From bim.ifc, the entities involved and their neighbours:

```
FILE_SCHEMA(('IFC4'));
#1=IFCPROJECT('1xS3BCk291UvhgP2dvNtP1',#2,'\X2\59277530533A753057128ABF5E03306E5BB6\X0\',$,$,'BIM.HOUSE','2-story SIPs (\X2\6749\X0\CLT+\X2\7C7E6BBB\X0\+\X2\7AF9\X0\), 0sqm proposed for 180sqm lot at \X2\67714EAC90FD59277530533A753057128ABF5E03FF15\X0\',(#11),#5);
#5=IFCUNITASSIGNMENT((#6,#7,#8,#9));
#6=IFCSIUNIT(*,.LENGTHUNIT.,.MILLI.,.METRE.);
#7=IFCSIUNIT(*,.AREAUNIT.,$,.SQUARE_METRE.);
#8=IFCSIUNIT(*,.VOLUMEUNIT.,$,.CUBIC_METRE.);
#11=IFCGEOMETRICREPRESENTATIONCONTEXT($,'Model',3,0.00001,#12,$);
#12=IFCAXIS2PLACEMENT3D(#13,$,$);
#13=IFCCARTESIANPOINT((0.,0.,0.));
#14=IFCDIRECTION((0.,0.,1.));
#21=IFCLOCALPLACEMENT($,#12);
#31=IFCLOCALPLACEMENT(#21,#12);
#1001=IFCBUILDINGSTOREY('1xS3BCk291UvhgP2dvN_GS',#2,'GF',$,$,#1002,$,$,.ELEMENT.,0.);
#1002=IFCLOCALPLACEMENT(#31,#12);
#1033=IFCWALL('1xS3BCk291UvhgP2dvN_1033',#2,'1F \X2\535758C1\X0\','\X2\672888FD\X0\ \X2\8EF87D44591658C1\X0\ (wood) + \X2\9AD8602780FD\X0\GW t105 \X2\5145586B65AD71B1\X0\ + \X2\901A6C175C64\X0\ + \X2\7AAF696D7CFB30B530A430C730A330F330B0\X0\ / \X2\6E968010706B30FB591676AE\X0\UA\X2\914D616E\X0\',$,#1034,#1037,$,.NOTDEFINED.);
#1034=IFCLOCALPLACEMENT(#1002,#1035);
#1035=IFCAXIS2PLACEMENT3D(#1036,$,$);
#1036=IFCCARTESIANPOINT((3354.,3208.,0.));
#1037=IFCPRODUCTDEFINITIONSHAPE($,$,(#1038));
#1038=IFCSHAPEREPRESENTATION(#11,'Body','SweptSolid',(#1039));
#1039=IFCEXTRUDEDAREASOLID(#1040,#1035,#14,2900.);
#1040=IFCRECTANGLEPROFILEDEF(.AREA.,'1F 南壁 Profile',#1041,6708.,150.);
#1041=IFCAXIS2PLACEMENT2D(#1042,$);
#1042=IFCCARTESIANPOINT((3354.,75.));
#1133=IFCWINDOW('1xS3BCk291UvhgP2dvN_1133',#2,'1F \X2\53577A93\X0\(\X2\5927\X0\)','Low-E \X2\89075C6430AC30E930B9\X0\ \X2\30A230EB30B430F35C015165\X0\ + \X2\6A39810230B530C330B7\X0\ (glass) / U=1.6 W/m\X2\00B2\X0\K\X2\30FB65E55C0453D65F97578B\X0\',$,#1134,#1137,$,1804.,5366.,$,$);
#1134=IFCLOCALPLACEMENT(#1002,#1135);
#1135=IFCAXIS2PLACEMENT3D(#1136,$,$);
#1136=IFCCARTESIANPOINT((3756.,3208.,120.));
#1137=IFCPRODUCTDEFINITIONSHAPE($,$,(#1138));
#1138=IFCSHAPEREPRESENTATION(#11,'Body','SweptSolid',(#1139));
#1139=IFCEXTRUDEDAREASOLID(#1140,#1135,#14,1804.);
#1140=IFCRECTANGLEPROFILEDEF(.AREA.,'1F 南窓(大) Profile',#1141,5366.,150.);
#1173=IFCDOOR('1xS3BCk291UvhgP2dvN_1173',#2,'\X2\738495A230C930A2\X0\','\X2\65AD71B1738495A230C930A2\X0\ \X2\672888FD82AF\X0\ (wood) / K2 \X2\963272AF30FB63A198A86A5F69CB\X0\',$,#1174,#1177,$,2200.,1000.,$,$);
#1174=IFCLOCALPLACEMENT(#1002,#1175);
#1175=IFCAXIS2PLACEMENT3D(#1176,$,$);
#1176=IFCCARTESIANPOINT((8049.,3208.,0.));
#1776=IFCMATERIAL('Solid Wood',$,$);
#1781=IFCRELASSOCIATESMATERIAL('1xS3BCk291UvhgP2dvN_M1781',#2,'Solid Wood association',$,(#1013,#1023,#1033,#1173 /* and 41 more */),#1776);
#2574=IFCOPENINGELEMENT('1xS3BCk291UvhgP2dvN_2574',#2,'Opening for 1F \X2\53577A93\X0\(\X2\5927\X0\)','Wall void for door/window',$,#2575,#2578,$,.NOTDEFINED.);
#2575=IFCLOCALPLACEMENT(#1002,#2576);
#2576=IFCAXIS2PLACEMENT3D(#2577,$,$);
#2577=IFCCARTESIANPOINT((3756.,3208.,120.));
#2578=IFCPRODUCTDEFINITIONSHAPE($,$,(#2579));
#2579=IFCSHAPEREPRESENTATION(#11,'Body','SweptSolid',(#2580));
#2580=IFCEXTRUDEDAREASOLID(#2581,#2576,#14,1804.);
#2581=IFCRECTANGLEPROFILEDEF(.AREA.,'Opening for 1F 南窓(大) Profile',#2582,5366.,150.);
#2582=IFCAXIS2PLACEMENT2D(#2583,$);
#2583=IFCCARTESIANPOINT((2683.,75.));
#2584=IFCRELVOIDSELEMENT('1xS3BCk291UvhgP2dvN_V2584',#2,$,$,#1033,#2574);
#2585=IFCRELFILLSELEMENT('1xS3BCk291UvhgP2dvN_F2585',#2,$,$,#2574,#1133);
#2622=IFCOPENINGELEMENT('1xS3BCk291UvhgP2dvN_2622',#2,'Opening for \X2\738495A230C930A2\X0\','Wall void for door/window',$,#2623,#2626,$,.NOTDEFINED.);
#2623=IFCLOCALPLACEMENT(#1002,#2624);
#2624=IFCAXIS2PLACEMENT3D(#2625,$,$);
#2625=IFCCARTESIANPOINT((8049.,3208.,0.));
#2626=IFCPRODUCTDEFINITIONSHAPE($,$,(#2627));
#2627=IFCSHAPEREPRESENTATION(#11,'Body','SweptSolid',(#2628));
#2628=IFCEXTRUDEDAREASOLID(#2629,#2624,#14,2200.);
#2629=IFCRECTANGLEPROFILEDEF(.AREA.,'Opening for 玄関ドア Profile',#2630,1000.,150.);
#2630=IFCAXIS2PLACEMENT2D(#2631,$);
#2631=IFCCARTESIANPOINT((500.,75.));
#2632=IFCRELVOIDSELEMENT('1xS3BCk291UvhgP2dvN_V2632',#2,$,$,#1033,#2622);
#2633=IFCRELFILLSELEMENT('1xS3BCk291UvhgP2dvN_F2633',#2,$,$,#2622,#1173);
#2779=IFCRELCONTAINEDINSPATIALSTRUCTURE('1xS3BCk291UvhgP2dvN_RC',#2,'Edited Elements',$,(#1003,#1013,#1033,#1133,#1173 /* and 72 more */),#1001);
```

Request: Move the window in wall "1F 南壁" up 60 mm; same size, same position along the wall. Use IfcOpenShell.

```python
import numpy as np
import ifcopenshell
import ifcopenshell.api.geometry
import ifcopenshell.util.placement
import ifcopenshell.util.unit

model = ifcopenshell.open("bim.ifc")
unit_scale = ifcopenshell.util.unit.calculate_unit_scale(model)

window = model.by_guid("1xS3BCk291UvhgP2dvN_1133")
opening = window.FillsVoids[0].RelatingOpeningElement
dz = 60.0

shift = np.array([0.0, 0.0, dz])
# The window is not placed relative to its opening, so move both.
for product in (opening, window):
    matrix = ifcopenshell.util.placement.get_local_placement(product.ObjectPlacement)
    matrix[:3, 3] += shift
    ifcopenshell.api.geometry.edit_object_placement(model, product=product, matrix=matrix, is_si=False)

print(f"moved by {dz * unit_scale:+.3f} m")

model.write("bim_rev.ifc")
```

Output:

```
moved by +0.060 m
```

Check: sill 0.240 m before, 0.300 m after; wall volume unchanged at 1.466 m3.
